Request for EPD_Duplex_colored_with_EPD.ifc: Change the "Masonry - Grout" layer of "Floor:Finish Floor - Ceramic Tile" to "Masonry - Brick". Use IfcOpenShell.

First a look at what the model holds.

```python
import ifcopenshell
import ifcopenshell.util.element

model = ifcopenshell.open("EPD_Duplex_colored_with_EPD.ifc")
print(model.schema)
for layer_set in model.by_type("IfcMaterialLayerSet"):
    if layer_set.LayerSetName == "Floor:Finish Floor - Ceramic Tile":
        for layer in layer_set.MaterialLayers:
            print(layer.id(), layer.Material and layer.Material.Name, layer.LayerThickness, sep=" | ")
        print(len(ifcopenshell.util.element.get_elements_by_material(model, layer_set)), "elements and types use it")
print(sorted(m.Name for m in model.by_type("IfcMaterial") if m.Name)[:60])
```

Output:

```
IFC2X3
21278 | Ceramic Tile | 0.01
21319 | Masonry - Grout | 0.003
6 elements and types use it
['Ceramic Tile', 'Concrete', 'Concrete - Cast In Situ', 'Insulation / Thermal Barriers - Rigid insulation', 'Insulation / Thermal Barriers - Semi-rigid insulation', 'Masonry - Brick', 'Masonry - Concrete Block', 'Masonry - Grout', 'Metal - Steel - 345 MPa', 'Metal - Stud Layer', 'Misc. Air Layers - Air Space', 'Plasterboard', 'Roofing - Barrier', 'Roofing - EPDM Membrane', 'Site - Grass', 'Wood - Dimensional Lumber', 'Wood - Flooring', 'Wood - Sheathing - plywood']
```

```python
import ifcopenshell
import ifcopenshell.api.material

model = ifcopenshell.open("EPD_Duplex_colored_with_EPD.ifc")

layer_set = next(s for s in model.by_type("IfcMaterialLayerSet") if s.LayerSetName == "Floor:Finish Floor - Ceramic Tile")
layer = next(l for l in layer_set.MaterialLayers if l.Material and l.Material.Name == "Masonry - Grout")
material = next(m for m in model.by_type("IfcMaterial") if m.Name == "Masonry - Brick")

# Point this one layer at the other material; renaming the old one would change it everywhere.
ifcopenshell.api.material.edit_layer(model, layer=layer, attributes={}, material=material)

print([l.Material.Name if l.Material else None for l in layer_set.MaterialLayers])

model.write("EPD_Duplex_colored_with_EPD_rev.ifc")
```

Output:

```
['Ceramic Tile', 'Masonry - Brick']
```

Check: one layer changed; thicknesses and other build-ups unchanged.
